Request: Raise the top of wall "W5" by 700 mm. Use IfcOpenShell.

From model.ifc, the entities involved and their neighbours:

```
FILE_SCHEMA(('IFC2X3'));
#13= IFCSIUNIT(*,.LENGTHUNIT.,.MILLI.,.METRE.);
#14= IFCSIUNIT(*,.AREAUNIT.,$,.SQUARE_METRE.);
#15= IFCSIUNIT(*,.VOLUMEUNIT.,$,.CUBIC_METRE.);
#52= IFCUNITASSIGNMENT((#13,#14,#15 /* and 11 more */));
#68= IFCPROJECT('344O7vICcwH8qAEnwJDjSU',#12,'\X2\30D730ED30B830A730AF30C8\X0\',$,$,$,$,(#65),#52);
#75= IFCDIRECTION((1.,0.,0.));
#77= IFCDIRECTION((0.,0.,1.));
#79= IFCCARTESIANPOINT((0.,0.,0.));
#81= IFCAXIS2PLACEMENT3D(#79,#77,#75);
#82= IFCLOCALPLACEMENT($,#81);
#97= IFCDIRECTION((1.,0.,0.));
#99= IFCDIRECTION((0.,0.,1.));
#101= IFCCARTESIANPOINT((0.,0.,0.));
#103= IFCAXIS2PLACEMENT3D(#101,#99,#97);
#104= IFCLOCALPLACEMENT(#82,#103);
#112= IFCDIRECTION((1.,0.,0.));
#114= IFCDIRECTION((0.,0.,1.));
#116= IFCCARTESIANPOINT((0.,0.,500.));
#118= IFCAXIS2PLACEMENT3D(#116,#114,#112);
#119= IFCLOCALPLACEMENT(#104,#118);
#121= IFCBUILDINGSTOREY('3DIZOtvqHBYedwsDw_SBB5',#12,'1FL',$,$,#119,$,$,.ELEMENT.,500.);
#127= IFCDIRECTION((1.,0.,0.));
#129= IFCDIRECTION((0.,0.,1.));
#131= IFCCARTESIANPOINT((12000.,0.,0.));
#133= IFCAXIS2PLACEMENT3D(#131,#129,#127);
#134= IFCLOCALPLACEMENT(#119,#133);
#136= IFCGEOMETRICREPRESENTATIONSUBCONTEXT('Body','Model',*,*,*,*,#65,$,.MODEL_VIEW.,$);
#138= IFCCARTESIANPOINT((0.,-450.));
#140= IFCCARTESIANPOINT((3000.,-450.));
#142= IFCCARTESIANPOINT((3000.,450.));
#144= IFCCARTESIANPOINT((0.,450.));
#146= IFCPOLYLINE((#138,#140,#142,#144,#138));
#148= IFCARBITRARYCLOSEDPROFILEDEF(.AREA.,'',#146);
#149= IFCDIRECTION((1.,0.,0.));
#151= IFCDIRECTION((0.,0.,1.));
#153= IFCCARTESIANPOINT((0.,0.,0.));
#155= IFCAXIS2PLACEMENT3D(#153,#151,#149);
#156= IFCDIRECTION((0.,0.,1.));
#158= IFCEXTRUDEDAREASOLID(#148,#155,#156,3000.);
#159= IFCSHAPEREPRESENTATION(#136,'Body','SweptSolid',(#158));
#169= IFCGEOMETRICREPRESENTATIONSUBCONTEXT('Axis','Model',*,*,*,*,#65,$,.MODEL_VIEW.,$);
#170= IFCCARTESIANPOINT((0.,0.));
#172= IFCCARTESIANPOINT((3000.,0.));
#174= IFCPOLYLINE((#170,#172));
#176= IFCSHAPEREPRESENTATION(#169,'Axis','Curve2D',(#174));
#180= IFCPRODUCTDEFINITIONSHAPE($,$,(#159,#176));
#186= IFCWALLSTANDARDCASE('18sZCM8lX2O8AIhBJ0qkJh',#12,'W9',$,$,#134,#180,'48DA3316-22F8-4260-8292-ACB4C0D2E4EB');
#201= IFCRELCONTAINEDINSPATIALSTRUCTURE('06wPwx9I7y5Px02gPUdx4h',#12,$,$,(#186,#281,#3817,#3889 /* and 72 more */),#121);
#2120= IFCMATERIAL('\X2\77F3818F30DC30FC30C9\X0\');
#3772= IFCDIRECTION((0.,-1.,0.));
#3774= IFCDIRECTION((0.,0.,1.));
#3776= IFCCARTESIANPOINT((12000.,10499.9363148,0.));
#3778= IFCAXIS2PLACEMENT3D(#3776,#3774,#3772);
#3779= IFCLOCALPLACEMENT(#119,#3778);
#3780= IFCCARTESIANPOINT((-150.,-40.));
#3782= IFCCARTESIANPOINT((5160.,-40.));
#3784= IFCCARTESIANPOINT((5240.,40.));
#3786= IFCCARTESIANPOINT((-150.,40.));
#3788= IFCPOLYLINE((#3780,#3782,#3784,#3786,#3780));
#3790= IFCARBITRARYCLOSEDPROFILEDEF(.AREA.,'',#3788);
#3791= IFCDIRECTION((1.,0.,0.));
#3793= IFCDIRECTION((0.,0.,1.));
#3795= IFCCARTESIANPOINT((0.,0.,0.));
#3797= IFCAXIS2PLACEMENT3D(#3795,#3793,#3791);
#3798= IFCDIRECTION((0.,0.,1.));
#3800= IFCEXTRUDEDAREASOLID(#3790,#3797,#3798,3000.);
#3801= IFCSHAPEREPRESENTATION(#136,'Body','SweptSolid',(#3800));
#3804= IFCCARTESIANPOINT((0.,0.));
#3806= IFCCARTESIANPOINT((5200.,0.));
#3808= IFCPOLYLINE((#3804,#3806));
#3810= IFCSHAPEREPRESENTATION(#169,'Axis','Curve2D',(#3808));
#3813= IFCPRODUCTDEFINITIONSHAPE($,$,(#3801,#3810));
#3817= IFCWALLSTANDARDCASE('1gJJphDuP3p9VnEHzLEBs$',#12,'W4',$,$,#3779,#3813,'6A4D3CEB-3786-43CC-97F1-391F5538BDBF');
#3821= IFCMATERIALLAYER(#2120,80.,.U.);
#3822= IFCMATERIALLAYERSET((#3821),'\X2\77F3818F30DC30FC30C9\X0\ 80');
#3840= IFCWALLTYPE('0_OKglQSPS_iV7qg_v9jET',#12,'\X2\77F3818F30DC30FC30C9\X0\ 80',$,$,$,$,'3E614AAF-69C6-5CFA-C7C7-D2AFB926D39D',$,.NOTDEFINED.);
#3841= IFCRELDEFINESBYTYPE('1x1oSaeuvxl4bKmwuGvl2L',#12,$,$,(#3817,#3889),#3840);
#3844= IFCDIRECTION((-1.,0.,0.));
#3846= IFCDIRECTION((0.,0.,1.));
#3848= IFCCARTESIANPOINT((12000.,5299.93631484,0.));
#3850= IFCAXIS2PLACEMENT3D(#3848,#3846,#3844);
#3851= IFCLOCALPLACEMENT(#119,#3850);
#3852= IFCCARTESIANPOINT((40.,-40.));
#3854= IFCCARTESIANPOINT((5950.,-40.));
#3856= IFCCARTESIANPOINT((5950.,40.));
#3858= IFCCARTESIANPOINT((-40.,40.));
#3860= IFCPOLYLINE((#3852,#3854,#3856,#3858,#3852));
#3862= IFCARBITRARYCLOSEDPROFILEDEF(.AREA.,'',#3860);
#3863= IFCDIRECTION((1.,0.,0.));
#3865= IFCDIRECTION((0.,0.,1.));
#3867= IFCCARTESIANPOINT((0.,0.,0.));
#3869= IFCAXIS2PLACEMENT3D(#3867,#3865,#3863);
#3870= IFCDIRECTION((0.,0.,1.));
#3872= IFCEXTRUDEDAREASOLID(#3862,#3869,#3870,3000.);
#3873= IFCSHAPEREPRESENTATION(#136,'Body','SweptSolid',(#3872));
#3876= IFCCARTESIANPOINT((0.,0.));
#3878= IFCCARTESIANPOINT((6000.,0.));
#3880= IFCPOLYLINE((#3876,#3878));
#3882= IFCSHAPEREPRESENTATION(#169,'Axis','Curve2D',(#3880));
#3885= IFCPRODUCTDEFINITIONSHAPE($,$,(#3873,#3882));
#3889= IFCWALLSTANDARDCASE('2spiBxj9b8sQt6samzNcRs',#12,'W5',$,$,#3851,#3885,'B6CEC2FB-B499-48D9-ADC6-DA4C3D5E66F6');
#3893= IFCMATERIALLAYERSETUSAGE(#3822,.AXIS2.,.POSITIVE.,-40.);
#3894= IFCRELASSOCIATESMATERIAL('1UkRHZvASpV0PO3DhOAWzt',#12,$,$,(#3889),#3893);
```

```python
import ifcopenshell
import ifcopenshell.geom
import ifcopenshell.util.representation
import ifcopenshell.util.shape

model = ifcopenshell.open("model.ifc")
settings = ifcopenshell.geom.settings()


def volume(element):
    """Net volume in cubic metres, openings subtracted."""
    shape = ifcopenshell.geom.create_shape(settings, element)
    return ifcopenshell.util.shape.get_volume(shape.geometry)


wall = model.by_guid("2spiBxj9b8sQt6samzNcRs")
before = volume(wall)

body = ifcopenshell.util.representation.get_representation(wall, "Model", "Body")
solid = body.Items[0]
old_height = solid.Depth
solid.Depth += 700.0
after = volume(wall)

print(f"height {old_height:g} -> {solid.Depth:g}, volume {before:.3f} -> {after:.3f} m3")

model.write("model-out.ifc")
```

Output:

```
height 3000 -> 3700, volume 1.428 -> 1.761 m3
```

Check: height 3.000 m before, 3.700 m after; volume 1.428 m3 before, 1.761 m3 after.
